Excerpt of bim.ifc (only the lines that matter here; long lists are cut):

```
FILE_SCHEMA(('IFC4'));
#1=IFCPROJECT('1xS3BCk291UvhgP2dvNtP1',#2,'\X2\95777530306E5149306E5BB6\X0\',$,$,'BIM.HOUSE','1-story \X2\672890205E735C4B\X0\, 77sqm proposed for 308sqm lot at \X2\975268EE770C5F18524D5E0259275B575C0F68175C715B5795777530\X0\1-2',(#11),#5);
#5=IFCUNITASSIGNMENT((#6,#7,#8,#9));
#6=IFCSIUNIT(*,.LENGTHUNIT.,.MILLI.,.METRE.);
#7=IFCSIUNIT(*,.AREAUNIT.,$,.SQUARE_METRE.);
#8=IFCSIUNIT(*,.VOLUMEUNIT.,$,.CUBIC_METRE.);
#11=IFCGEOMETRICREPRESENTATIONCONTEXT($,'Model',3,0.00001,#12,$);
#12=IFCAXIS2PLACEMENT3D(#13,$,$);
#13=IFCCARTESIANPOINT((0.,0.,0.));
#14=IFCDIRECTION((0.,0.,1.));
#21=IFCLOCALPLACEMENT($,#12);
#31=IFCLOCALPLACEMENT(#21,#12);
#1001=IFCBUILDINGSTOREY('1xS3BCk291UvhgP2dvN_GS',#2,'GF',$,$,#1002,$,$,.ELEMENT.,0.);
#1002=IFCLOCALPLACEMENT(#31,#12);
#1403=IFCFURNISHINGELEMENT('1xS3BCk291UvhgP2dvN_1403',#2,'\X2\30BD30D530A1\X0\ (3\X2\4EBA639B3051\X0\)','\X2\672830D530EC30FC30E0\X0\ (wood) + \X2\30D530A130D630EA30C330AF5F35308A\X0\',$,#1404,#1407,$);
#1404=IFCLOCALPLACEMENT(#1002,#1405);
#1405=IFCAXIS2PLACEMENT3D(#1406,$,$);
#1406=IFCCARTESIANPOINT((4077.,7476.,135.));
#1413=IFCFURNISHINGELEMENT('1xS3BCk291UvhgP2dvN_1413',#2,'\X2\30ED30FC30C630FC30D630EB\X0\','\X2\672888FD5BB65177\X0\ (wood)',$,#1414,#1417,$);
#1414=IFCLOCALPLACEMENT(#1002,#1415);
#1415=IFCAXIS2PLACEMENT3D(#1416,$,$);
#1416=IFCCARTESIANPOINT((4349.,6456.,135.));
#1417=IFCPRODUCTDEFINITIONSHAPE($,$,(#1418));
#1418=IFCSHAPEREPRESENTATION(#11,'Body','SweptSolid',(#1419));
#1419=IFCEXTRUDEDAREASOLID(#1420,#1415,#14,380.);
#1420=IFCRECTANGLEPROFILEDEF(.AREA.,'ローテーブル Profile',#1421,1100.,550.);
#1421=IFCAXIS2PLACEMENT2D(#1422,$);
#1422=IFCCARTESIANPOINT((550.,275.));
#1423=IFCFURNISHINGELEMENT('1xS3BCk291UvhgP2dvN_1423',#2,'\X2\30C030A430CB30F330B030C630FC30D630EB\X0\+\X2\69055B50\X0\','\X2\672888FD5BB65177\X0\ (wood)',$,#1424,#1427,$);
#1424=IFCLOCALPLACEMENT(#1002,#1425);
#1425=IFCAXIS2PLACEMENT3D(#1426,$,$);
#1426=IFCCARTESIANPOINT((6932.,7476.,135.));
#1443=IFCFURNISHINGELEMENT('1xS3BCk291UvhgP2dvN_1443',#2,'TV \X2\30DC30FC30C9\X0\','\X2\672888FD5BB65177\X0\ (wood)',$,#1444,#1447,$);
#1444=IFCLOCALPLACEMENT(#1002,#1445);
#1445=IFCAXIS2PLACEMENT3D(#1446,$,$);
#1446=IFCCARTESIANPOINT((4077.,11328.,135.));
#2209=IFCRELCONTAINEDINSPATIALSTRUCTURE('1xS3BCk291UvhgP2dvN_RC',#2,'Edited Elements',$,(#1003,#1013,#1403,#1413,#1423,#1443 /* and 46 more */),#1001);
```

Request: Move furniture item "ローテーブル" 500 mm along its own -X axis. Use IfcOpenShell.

```python
import ifcopenshell
import ifcopenshell.api.geometry
import ifcopenshell.util.placement
import ifcopenshell.util.unit

model = ifcopenshell.open("bim.ifc")
unit_scale = ifcopenshell.util.unit.calculate_unit_scale(model)

item = model.by_guid("1xS3BCk291UvhgP2dvN_1413")
matrix = ifcopenshell.util.placement.get_local_placement(item.ObjectPlacement)
matrix[:3, 3] -= matrix[:3, 0] * 0.5 / unit_scale
ifcopenshell.api.geometry.edit_object_placement(model, product=item, matrix=matrix, is_si=False)

print(ifcopenshell.util.placement.get_local_placement(item.ObjectPlacement).round(3) + 0.0)

model.write("bim-out.ifc")
```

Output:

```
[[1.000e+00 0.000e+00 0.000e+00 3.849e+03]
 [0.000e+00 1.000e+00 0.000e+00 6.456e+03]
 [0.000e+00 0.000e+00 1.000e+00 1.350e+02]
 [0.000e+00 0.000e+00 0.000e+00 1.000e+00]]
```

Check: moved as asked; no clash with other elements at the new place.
